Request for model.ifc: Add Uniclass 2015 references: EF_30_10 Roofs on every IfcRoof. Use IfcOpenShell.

First a look at what the model holds.

```python
import ifcopenshell

model = ifcopenshell.open("model.ifc")
print(model.schema)
print("classifications:", [c.Name for c in model.by_type("IfcClassification")])
for ifc_class in ("IfcDoor", "IfcRoof", "IfcStair", "IfcWall", "IfcWindow"):
    print(ifc_class, len(model.by_type(ifc_class)))
```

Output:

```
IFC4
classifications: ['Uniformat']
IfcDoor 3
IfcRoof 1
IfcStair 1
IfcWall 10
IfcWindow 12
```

```python
import ifcopenshell
import ifcopenshell.api.classification

model = ifcopenshell.open("model.ifc")

system = ifcopenshell.api.classification.add_classification(model, classification="Uniclass 2015")

codes = {
    "IfcRoof": ("EF_30_10", "Roofs"),
}
for ifc_class, (code, name) in codes.items():
    products = model.by_type(ifc_class)
    ifcopenshell.api.classification.add_reference(
        model, products=products, classification=system, identification=code, name=name
    )
    print(code, len(products))

model.write("model_updated.ifc")
```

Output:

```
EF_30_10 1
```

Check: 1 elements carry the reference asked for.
